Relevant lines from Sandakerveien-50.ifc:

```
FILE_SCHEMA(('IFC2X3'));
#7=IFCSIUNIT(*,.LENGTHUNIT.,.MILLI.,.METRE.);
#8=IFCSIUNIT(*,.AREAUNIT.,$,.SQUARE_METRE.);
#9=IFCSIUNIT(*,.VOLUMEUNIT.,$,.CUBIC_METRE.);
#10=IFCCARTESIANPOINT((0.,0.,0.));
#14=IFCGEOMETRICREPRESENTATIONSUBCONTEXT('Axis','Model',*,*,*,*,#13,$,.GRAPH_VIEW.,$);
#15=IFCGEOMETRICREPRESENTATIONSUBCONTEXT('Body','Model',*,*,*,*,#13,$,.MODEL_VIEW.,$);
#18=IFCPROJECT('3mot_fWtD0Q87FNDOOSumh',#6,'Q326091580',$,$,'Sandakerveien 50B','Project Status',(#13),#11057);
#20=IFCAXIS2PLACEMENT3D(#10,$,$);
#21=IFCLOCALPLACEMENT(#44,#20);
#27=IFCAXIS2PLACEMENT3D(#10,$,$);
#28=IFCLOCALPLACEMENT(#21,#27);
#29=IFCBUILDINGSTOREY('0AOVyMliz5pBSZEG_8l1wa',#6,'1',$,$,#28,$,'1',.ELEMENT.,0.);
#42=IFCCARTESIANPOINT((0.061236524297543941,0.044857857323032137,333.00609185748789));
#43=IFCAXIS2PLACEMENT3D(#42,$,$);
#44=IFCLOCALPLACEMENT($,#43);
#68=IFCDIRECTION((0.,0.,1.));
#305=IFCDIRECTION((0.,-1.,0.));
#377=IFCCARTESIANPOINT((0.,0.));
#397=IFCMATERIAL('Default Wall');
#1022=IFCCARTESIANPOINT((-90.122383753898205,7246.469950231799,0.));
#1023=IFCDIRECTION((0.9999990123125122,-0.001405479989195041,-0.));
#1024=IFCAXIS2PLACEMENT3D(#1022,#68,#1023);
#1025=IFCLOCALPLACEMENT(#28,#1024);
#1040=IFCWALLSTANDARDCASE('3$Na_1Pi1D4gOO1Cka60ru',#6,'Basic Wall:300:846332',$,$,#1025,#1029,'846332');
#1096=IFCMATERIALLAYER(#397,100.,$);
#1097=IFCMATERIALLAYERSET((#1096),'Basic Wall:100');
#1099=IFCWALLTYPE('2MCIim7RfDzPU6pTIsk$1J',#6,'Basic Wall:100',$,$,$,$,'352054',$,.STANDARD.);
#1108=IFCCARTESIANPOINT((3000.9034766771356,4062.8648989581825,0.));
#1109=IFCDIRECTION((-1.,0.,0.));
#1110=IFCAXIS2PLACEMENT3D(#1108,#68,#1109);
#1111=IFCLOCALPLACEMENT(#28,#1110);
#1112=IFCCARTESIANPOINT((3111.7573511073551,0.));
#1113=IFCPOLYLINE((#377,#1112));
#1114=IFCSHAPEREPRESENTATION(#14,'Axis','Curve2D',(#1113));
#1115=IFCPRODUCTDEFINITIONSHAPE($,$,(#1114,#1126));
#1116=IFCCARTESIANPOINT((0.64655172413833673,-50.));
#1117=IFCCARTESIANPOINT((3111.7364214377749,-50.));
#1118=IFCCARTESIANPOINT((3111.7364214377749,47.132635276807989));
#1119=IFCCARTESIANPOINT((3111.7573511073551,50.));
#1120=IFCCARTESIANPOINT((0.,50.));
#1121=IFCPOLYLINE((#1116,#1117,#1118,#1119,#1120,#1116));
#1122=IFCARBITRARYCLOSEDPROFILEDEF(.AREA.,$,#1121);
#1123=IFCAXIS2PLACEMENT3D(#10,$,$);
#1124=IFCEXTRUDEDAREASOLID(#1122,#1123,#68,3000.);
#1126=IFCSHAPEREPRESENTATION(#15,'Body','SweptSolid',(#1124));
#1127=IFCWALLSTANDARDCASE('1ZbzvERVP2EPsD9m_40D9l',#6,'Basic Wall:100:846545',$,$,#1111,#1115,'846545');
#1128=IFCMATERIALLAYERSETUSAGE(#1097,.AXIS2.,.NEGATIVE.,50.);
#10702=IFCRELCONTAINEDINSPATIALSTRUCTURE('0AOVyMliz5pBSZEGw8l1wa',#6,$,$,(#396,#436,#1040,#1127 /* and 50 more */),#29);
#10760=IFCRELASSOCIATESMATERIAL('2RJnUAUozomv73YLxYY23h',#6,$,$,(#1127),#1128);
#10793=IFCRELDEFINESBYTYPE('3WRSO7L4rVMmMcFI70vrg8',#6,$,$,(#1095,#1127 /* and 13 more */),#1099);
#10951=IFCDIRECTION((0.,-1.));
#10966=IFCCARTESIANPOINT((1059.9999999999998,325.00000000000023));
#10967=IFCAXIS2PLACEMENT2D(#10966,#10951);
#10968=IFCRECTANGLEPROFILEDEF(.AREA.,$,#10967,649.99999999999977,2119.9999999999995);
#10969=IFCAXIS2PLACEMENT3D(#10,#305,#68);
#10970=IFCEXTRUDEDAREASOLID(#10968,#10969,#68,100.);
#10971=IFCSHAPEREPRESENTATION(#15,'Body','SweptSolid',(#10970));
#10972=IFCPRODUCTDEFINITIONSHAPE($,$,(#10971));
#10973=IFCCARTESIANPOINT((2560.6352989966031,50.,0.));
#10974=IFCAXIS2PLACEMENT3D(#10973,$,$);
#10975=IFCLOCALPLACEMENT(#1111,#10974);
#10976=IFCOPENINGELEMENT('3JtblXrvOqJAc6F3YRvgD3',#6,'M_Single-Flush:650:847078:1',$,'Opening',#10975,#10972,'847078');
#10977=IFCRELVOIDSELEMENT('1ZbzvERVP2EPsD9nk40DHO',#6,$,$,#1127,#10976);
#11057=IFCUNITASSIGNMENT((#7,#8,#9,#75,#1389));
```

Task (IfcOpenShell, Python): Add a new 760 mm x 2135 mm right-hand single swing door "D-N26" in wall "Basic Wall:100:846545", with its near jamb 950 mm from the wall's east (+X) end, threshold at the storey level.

```python
import numpy as np
import ifcopenshell
import ifcopenshell.api.feature
import ifcopenshell.api.geometry
import ifcopenshell.api.root
import ifcopenshell.api.spatial
import ifcopenshell.api.type
import ifcopenshell.geom
import ifcopenshell.util.element
import ifcopenshell.util.placement
import ifcopenshell.util.representation
import ifcopenshell.util.shape
import ifcopenshell.util.unit

model = ifcopenshell.open("Sandakerveien-50.ifc")
unit_scale = ifcopenshell.util.unit.calculate_unit_scale(model)
settings = ifcopenshell.geom.settings()


def volume(element):
    """Net volume in cubic metres, openings subtracted."""
    shape = ifcopenshell.geom.create_shape(settings, element)
    return ifcopenshell.util.shape.get_volume(shape.geometry)


wall = model.by_guid("1ZbzvERVP2EPsD9m_40D9l")
storey = ifcopenshell.util.element.get_container(wall, ifc_class="IfcBuildingStorey")
context = ifcopenshell.util.representation.get_context(model, "Model", "Body", "MODEL_VIEW")
before = volume(wall)

width, height, from_end, sill = 0.76, 2.135, 0.95, 0.0  # metres

# The wall runs along its own X axis, and the end named is its -X end.
wall_shape = ifcopenshell.geom.create_shape(settings, wall)
x, y, z = ifcopenshell.util.shape.get_vertices(wall_shape.geometry).T
start = x.min() + from_end
face, thickness = float(y.min()), float(y.max() - y.min())
wall_matrix = ifcopenshell.util.placement.get_local_placement(wall.ObjectPlacement)
level = ifcopenshell.util.placement.get_local_placement(storey.ObjectPlacement)[2, 3]


def in_wall(x, y):
    """Placement at x, y metres in the wall's axes, at sill height."""
    matrix = wall_matrix.copy()
    matrix[:, 3] = wall_matrix @ np.array([x / unit_scale, y / unit_scale, 0.0, 1.0])
    matrix[2, 3] = level + sill / unit_scale
    return matrix


# Opening: a box that overshoots both wall faces by 50 mm.
opening = ifcopenshell.api.root.create_entity(model, ifc_class="IfcOpeningElement")
box = ifcopenshell.api.geometry.add_wall_representation(
    model, context=context, length=width, height=height, thickness=thickness + 0.1
)
ifcopenshell.api.geometry.assign_representation(model, product=opening, representation=box)
ifcopenshell.api.geometry.edit_object_placement(model, product=opening, matrix=in_wall(start, face - 0.05), is_si=False)
ifcopenshell.api.feature.add_feature(model, feature=opening, element=wall)

door = ifcopenshell.api.root.create_entity(model, ifc_class="IfcDoor", name="D-N26")
door.OverallWidth, door.OverallHeight = width / unit_scale, height / unit_scale
body = ifcopenshell.api.geometry.add_door_representation(
    model,
    context=context,
    overall_width=door.OverallWidth,
    overall_height=door.OverallHeight,
    operation_type="SINGLE_SWING_RIGHT",
    lining_properties={"LiningDepth": thickness / unit_scale, "ThresholdDepth": thickness / unit_scale},
)
ifcopenshell.api.geometry.assign_representation(model, product=door, representation=body)
ifcopenshell.api.spatial.assign_container(model, products=[door], relating_structure=storey)
fills = ifcopenshell.api.feature.add_filling(model, opening=opening, element=door)
fills.OwnerHistory = door.OwnerHistory  # required in IFC2X3

# IFC2X3 keeps the operation on the door style.
style = ifcopenshell.api.root.create_entity(model, ifc_class="IfcDoorStyle", name="D-N26")
style.OperationType, style.ConstructionType = "SINGLE_SWING_RIGHT", "NOTDEFINED"
style.ParameterTakesPrecedence = style.Sizeable = False
ifcopenshell.api.type.assign_type(model, related_objects=[door], relating_type=style)

# The lining spans the wall, so the door starts at the wall face.
ifcopenshell.api.geometry.edit_object_placement(model, product=door, matrix=in_wall(start, face), is_si=False)

after = volume(wall)

print(f"wall volume {before:.3f} -> {after:.3f} m3")

model.write("Sandakerveien-50_v2.ifc")
```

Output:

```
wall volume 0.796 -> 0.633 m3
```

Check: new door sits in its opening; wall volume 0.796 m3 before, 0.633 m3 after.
